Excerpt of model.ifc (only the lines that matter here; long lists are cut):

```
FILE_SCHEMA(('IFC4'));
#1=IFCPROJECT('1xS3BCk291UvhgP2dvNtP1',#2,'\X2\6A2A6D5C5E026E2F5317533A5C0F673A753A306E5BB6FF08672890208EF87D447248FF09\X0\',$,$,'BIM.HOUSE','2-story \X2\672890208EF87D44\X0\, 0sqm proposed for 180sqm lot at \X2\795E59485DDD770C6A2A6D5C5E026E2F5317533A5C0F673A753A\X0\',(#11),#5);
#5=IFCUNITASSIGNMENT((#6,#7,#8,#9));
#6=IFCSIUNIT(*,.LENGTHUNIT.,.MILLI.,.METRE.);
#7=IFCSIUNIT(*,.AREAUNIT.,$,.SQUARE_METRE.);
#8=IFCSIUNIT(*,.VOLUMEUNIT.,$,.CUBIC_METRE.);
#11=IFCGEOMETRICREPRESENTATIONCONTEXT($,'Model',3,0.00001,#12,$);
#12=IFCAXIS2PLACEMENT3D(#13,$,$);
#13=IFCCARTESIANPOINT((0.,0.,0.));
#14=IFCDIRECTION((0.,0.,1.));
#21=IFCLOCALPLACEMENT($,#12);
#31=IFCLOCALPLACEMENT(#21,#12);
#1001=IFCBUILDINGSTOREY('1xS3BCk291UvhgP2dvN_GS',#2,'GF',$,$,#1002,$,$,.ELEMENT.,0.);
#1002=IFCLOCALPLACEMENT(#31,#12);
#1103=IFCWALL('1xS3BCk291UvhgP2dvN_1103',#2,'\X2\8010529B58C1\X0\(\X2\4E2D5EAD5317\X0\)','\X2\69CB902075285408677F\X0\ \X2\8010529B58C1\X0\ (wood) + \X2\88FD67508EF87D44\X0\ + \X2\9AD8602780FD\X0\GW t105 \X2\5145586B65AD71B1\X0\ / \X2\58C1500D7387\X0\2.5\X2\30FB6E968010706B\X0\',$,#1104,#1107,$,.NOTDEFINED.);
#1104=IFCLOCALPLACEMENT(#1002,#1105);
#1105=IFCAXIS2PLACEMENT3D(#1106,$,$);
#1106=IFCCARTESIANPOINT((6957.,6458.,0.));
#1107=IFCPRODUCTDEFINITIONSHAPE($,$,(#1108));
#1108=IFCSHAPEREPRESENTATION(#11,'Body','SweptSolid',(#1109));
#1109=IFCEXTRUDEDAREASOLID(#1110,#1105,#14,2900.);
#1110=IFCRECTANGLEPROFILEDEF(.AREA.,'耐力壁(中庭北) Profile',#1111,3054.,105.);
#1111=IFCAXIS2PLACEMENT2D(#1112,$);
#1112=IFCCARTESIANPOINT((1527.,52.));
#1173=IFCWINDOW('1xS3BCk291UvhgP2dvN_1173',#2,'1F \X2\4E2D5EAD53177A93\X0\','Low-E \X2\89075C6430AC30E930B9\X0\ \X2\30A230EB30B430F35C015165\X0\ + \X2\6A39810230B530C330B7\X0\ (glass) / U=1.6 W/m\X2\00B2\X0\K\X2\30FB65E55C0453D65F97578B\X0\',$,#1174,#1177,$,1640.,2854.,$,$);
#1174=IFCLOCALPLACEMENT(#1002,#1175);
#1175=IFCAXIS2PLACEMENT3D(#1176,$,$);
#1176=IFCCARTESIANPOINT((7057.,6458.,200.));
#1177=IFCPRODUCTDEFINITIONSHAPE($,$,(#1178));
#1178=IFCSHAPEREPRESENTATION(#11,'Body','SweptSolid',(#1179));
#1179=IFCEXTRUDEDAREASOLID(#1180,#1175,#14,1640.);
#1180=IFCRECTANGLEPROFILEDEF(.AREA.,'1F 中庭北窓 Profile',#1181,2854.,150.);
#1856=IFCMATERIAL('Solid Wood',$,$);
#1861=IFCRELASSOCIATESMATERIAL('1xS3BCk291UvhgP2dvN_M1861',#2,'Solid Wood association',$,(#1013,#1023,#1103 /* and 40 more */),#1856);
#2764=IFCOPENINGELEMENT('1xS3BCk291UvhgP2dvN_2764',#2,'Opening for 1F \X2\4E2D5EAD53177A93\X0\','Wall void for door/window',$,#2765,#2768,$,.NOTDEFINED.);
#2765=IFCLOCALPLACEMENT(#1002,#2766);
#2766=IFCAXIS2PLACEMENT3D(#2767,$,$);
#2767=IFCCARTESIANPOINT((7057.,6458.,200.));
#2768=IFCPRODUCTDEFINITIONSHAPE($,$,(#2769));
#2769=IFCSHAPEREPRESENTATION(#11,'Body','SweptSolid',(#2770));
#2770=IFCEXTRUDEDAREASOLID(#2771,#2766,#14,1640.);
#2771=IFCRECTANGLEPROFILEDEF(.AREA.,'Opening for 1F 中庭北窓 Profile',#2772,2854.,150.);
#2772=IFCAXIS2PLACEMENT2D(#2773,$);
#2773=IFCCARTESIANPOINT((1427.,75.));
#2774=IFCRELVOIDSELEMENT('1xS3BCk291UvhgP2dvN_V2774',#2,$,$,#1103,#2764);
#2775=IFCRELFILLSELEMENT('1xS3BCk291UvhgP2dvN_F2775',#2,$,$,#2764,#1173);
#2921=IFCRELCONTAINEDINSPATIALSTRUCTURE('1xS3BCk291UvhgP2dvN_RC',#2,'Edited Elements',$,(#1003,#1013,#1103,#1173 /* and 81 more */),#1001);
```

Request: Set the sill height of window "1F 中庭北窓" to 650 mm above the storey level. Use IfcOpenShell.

```python
import numpy as np
import ifcopenshell
import ifcopenshell.api.geometry
import ifcopenshell.geom
import ifcopenshell.util.element
import ifcopenshell.util.placement
import ifcopenshell.util.shape
import ifcopenshell.util.unit

model = ifcopenshell.open("model.ifc")
unit_scale = ifcopenshell.util.unit.calculate_unit_scale(model)

window = model.by_id(1173)
opening = window.FillsVoids[0].RelatingOpeningElement
storey = ifcopenshell.util.element.get_container(window, ifc_class="IfcBuildingStorey")
level = ifcopenshell.util.placement.get_local_placement(storey.ObjectPlacement)[2, 3]

# The opening's origin need not be at the sill, so measure its lowest point.
shape = ifcopenshell.geom.create_shape(ifcopenshell.geom.settings(), opening)
bottom = ifcopenshell.util.shape.get_shape_bottom_elevation(shape, shape.geometry) / unit_scale
dz = level + 0.65 / unit_scale - bottom

shift = np.array([0.0, 0.0, dz])
# The window is not placed relative to its opening, so move both.
for product in (opening, window):
    matrix = ifcopenshell.util.placement.get_local_placement(product.ObjectPlacement)
    matrix[:3, 3] += shift
    ifcopenshell.api.geometry.edit_object_placement(model, product=product, matrix=matrix, is_si=False)

print(f"moved by {dz * unit_scale:+.3f} m")

model.write("model_v2.ifc")
```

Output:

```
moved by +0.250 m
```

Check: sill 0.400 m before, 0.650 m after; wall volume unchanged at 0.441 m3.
